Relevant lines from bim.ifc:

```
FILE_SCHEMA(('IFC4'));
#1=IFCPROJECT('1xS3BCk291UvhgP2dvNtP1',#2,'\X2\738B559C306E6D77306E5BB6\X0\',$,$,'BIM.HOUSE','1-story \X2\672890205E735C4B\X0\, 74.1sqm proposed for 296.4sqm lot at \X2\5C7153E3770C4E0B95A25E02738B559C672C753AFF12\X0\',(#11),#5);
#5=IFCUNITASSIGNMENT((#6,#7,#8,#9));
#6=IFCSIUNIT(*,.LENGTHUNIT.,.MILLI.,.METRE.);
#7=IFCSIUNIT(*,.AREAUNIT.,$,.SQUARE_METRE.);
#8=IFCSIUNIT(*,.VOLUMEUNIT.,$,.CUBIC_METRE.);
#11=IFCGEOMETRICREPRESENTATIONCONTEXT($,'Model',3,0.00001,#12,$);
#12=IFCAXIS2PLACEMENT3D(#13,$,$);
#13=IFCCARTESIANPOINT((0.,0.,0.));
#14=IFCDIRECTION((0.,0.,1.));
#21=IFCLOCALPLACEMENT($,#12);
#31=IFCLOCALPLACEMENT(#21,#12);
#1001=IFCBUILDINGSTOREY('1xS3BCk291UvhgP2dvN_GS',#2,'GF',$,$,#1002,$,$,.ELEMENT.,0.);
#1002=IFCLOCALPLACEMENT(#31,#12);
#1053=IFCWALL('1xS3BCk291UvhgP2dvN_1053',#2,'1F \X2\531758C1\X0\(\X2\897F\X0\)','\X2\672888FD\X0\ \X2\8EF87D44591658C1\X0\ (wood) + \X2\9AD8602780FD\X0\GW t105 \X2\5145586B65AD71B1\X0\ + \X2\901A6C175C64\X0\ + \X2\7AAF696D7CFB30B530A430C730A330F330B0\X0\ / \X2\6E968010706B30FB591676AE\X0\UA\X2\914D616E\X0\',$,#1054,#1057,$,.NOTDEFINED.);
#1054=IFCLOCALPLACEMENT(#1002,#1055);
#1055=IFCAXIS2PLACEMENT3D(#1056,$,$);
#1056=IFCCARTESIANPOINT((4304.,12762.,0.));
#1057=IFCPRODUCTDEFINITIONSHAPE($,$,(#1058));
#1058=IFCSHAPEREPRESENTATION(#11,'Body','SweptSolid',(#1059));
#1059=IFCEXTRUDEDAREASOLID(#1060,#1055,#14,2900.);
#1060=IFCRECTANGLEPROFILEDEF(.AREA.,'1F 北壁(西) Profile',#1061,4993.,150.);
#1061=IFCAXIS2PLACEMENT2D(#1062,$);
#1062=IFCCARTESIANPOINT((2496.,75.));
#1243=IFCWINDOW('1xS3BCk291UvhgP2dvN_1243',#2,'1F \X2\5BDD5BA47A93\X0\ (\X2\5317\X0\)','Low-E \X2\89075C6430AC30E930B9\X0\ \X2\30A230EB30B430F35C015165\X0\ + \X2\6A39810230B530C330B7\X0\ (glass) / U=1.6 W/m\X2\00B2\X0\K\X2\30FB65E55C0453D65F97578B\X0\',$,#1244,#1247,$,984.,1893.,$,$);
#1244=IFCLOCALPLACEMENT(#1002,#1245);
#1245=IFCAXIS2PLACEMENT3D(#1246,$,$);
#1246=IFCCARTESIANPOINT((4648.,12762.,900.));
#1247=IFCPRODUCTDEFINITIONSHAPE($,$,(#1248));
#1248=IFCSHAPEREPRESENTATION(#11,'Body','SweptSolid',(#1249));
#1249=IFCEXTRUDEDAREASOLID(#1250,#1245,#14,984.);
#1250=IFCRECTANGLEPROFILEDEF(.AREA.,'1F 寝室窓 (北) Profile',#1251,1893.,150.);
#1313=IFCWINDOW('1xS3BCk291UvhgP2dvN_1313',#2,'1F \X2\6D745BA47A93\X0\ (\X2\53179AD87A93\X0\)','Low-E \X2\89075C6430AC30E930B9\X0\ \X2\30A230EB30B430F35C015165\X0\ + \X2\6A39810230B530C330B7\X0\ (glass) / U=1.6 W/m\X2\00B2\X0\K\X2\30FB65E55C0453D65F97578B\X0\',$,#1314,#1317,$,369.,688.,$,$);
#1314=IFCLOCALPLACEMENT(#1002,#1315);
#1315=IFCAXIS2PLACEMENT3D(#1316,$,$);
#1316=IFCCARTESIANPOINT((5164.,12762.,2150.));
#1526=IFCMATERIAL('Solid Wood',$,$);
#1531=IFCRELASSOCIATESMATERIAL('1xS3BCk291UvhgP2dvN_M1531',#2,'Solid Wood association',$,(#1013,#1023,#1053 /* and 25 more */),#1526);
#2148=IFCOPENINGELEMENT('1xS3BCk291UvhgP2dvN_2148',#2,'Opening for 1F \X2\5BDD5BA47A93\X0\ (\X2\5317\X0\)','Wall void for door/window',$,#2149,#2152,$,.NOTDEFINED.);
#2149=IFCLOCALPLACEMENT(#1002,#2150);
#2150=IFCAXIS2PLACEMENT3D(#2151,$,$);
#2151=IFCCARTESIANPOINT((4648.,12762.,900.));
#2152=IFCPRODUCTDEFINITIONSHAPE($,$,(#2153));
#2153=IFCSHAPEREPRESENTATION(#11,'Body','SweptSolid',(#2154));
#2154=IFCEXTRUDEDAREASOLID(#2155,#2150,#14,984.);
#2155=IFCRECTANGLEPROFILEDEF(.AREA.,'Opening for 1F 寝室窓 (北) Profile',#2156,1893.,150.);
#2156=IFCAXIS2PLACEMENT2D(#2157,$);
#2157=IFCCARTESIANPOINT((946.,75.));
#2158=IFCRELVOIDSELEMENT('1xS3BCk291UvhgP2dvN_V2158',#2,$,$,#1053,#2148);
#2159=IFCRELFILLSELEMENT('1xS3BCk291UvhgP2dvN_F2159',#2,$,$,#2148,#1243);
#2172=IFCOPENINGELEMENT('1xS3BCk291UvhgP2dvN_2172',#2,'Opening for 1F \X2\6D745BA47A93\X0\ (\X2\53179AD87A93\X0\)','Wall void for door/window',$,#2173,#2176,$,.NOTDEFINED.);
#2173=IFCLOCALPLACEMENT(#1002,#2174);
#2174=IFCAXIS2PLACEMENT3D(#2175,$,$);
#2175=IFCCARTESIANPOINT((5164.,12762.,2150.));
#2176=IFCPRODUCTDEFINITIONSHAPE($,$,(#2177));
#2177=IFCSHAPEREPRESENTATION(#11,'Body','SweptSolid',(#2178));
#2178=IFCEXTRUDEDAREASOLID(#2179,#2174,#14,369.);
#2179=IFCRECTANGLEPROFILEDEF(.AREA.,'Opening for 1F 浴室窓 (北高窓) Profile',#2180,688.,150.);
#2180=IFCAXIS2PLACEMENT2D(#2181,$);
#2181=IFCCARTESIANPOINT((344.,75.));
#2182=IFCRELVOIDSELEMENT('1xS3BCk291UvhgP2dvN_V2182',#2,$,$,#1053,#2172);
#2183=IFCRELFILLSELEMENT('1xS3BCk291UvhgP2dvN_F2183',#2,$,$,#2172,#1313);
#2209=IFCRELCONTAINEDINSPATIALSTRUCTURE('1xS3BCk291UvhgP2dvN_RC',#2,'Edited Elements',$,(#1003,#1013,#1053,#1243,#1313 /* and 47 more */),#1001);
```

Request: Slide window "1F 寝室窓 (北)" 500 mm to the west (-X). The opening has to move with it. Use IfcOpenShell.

```python
import ifcopenshell
import ifcopenshell.api.geometry
import ifcopenshell.util.placement
import ifcopenshell.util.unit

model = ifcopenshell.open("bim.ifc")
unit_scale = ifcopenshell.util.unit.calculate_unit_scale(model)

window = model.by_guid("1xS3BCk291UvhgP2dvN_1243")
opening = window.FillsVoids[0].RelatingOpeningElement
wall = opening.VoidsElements[0].RelatingBuildingElement

wall_matrix = ifcopenshell.util.placement.get_local_placement(wall.ObjectPlacement)
shift = wall_matrix[:3, 0] * -0.5 / unit_scale
before = ifcopenshell.util.placement.get_local_placement(window.ObjectPlacement)[:3, 3].copy()

# The window is not placed relative to its opening, so move both.
for product in (opening, window):
    matrix = ifcopenshell.util.placement.get_local_placement(product.ObjectPlacement)
    matrix[:3, 3] += shift
    ifcopenshell.api.geometry.edit_object_placement(model, product=product, matrix=matrix, is_si=False)

after = ifcopenshell.util.placement.get_local_placement(window.ObjectPlacement)[:3, 3]
print("window moved by", (after - before).round(3) + 0.0)

model.write("bim_updated.ifc")
```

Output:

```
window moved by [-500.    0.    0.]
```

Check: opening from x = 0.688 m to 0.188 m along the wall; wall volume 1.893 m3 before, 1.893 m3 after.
